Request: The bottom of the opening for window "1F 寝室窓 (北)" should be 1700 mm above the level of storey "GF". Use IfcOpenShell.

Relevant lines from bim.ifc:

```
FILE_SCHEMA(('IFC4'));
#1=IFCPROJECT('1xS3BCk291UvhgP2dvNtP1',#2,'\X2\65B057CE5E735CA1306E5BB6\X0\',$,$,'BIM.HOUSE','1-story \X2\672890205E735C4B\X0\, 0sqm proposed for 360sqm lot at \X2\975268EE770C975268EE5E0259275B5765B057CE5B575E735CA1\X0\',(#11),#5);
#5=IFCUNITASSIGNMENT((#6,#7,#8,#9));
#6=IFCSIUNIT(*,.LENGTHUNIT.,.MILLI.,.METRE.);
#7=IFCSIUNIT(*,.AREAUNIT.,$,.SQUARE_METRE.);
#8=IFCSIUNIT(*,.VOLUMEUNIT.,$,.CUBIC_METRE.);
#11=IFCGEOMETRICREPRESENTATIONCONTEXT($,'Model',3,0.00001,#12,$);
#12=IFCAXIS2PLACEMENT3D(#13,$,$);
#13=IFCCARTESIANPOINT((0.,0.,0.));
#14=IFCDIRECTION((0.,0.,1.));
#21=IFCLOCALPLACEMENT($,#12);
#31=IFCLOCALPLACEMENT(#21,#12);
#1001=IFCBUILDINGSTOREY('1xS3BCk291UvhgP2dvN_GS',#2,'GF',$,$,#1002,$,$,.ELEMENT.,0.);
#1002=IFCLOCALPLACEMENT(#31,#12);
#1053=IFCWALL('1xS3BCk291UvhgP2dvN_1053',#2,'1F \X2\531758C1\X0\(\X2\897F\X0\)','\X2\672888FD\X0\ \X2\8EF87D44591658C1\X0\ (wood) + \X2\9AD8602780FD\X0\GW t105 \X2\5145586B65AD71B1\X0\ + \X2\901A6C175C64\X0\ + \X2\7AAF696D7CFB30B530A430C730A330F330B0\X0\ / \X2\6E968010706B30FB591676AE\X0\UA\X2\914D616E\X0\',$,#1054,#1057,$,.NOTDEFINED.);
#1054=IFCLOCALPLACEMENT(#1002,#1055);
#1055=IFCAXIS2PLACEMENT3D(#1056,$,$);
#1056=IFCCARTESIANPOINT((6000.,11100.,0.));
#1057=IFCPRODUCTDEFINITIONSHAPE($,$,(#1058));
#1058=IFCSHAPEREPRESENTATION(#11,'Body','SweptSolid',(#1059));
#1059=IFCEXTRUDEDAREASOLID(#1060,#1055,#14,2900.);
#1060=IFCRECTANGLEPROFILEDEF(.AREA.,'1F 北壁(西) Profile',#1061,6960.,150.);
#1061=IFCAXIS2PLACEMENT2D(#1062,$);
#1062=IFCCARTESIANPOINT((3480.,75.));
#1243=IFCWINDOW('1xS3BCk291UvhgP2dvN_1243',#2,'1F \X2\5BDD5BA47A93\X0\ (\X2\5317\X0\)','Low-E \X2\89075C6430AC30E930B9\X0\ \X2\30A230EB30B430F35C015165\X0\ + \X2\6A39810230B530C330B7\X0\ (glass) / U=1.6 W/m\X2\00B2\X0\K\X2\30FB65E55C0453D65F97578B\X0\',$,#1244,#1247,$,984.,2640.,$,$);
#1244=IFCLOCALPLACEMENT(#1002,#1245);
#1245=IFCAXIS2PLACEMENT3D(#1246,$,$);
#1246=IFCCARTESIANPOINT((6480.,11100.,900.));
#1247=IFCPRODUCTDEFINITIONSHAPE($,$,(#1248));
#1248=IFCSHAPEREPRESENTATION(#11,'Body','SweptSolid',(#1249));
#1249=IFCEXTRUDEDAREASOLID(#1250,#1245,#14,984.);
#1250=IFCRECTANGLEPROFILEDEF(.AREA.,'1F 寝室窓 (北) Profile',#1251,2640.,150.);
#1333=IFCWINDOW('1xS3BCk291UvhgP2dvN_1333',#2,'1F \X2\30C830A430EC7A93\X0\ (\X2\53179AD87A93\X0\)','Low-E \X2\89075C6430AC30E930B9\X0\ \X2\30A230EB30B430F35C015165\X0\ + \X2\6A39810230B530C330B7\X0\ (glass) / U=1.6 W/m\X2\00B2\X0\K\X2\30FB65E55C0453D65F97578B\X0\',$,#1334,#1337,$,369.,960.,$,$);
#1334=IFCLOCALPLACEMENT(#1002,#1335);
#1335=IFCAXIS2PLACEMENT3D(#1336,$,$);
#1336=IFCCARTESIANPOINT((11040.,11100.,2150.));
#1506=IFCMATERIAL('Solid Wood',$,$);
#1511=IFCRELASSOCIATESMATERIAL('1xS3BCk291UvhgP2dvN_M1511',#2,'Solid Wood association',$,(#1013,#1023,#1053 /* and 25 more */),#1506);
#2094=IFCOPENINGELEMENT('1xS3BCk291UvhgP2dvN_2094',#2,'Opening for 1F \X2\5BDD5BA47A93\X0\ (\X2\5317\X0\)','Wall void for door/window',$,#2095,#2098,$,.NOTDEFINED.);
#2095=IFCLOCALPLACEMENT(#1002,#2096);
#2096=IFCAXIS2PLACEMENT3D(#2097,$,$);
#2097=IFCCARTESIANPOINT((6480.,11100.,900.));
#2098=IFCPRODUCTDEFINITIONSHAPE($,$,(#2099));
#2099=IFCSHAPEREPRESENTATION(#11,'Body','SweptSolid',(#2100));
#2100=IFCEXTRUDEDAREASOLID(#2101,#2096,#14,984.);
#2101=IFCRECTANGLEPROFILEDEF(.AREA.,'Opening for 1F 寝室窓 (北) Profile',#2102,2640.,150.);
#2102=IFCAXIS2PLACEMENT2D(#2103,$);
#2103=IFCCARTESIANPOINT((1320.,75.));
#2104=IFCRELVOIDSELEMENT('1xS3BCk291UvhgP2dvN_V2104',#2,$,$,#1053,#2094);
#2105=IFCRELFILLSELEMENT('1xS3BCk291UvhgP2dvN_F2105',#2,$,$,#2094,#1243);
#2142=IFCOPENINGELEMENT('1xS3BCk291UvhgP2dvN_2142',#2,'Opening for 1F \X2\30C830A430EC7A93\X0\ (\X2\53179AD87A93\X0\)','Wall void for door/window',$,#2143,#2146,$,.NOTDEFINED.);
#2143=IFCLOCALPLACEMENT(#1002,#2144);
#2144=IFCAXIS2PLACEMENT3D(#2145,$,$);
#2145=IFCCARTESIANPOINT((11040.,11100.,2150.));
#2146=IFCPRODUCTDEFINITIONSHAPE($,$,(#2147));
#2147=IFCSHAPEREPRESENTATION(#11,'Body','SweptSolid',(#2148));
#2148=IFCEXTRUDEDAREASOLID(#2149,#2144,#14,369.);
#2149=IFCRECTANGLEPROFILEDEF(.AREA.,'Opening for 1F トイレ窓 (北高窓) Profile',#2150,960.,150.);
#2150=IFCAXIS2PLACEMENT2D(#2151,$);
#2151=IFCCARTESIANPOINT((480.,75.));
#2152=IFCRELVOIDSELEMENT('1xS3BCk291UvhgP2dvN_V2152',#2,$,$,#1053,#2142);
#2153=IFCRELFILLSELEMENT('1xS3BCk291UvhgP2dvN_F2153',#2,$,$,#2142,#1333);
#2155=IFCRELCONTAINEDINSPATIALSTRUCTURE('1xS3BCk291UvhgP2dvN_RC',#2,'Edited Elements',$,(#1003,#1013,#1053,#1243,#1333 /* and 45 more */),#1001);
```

```python
import numpy as np
import ifcopenshell
import ifcopenshell.api.geometry
import ifcopenshell.geom
import ifcopenshell.util.element
import ifcopenshell.util.placement
import ifcopenshell.util.shape
import ifcopenshell.util.unit

model = ifcopenshell.open("bim.ifc")
unit_scale = ifcopenshell.util.unit.calculate_unit_scale(model)

window = model.by_guid("1xS3BCk291UvhgP2dvN_1243")
opening = window.FillsVoids[0].RelatingOpeningElement
storey = ifcopenshell.util.element.get_container(window, ifc_class="IfcBuildingStorey")
level = ifcopenshell.util.placement.get_local_placement(storey.ObjectPlacement)[2, 3]

# The opening's origin need not be at the sill, so measure its lowest point.
shape = ifcopenshell.geom.create_shape(ifcopenshell.geom.settings(), opening)
bottom = ifcopenshell.util.shape.get_shape_bottom_elevation(shape, shape.geometry) / unit_scale
dz = level + 1.7 / unit_scale - bottom

shift = np.array([0.0, 0.0, dz])
# The window is not placed relative to its opening, so move both.
for product in (opening, window):
    matrix = ifcopenshell.util.placement.get_local_placement(product.ObjectPlacement)
    matrix[:3, 3] += shift
    ifcopenshell.api.geometry.edit_object_placement(model, product=product, matrix=matrix, is_si=False)

print(f"moved by {dz * unit_scale:+.3f} m")

model.write("bim_rev.ifc")
```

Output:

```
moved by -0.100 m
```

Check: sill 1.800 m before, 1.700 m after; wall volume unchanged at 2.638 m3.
